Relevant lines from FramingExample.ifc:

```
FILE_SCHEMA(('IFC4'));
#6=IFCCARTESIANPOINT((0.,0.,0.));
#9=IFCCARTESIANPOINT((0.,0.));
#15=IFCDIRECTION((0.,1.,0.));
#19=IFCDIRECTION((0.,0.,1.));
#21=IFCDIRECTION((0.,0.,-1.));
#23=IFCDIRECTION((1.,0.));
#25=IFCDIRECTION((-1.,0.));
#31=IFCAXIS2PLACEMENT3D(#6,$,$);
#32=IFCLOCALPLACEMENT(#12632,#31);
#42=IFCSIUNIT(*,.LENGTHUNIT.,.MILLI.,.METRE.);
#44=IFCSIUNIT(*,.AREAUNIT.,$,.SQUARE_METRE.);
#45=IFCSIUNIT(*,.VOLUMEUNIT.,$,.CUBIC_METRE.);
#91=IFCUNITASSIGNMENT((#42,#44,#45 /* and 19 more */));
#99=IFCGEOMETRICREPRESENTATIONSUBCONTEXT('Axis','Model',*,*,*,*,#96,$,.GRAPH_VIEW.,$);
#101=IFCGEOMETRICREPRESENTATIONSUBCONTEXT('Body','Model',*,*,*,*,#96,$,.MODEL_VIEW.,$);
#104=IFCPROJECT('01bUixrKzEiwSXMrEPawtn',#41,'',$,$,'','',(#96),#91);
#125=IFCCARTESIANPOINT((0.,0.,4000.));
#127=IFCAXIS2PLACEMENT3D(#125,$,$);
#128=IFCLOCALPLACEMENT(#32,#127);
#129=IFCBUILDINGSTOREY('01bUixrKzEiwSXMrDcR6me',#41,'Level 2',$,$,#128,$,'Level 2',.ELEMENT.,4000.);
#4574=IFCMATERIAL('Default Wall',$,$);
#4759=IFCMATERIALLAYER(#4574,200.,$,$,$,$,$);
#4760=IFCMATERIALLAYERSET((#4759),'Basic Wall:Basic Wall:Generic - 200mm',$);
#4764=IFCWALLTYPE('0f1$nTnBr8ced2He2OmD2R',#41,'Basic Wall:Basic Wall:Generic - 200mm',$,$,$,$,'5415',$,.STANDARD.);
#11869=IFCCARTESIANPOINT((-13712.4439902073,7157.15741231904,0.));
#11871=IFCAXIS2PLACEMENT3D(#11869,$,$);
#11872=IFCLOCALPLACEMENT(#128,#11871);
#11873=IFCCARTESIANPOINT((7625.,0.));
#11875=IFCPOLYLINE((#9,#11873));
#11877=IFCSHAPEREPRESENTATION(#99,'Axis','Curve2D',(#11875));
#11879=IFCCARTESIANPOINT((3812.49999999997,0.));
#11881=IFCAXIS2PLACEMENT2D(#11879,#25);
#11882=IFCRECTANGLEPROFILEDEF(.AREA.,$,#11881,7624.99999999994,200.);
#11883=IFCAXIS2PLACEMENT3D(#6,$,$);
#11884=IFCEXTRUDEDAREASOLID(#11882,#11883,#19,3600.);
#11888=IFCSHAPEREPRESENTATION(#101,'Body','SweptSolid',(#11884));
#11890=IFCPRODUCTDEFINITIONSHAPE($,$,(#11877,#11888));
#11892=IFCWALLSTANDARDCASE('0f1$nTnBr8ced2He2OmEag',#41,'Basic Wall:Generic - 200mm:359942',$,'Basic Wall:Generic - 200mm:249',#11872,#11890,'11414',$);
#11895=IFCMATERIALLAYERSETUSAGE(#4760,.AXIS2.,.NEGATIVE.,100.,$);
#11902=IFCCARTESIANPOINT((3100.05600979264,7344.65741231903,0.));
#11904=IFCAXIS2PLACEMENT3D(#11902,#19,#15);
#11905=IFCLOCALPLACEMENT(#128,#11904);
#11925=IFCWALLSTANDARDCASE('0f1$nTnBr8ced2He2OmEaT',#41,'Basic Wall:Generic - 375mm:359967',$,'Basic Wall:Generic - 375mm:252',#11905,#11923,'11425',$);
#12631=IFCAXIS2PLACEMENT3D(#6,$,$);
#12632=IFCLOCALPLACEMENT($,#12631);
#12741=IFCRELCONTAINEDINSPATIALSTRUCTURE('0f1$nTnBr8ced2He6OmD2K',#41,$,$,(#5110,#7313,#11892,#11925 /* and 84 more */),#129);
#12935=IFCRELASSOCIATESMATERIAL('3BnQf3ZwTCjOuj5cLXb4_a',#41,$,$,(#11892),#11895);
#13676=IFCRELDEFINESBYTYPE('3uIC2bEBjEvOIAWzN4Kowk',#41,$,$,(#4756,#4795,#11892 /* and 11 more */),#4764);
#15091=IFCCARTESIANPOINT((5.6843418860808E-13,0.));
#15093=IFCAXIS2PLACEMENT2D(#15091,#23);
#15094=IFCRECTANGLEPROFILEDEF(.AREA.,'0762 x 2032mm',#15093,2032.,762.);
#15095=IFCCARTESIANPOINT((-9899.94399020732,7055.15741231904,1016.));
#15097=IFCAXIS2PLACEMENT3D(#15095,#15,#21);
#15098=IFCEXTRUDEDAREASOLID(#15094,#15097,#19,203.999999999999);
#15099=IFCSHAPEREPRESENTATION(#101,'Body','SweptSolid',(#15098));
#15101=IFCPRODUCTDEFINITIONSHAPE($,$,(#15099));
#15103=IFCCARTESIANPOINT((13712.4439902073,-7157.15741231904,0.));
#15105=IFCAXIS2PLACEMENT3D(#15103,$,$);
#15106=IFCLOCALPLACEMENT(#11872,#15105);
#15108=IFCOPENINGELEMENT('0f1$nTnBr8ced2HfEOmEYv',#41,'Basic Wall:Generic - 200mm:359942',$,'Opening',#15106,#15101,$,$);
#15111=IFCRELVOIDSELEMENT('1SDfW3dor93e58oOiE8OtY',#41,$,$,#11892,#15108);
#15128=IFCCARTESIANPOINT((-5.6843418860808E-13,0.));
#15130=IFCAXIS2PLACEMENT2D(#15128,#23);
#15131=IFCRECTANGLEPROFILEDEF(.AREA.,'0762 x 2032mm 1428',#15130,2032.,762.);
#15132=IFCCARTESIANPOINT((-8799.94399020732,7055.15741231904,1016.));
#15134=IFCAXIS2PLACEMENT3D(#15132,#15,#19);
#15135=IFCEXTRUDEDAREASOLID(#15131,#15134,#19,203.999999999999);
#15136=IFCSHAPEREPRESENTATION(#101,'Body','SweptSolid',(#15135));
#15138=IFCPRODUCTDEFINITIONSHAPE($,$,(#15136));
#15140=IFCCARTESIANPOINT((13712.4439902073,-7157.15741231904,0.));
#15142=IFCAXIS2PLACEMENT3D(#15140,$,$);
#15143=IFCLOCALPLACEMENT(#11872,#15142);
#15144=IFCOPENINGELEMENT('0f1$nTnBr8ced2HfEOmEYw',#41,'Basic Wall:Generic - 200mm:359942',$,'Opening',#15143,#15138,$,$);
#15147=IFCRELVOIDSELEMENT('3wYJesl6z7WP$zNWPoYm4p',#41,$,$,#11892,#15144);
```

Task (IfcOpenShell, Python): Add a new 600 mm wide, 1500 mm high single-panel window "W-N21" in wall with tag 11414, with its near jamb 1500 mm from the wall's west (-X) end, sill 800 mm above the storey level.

```python
import numpy as np
import ifcopenshell
import ifcopenshell.api.feature
import ifcopenshell.api.geometry
import ifcopenshell.api.root
import ifcopenshell.api.spatial
import ifcopenshell.geom
import ifcopenshell.util.element
import ifcopenshell.util.placement
import ifcopenshell.util.representation
import ifcopenshell.util.shape
import ifcopenshell.util.unit

model = ifcopenshell.open("FramingExample.ifc")
unit_scale = ifcopenshell.util.unit.calculate_unit_scale(model)
settings = ifcopenshell.geom.settings()


def volume(element):
    """Net volume in cubic metres, openings subtracted."""
    shape = ifcopenshell.geom.create_shape(settings, element)
    return ifcopenshell.util.shape.get_volume(shape.geometry)


wall = model.by_guid("0f1$nTnBr8ced2He2OmEag")
storey = ifcopenshell.util.element.get_container(wall, ifc_class="IfcBuildingStorey")
context = ifcopenshell.util.representation.get_context(model, "Model", "Body", "MODEL_VIEW")
before = volume(wall)

width, height, from_end, sill = 0.6, 1.5, 1.5, 0.8  # metres

# The wall runs along its own X axis, and the end named is its -X end.
wall_shape = ifcopenshell.geom.create_shape(settings, wall)
x, y, z = ifcopenshell.util.shape.get_vertices(wall_shape.geometry).T
start = x.min() + from_end
face, thickness = float(y.min()), float(y.max() - y.min())
wall_matrix = ifcopenshell.util.placement.get_local_placement(wall.ObjectPlacement)
level = ifcopenshell.util.placement.get_local_placement(storey.ObjectPlacement)[2, 3]


def in_wall(x, y):
    """Placement at x, y metres in the wall's axes, at sill height."""
    matrix = wall_matrix.copy()
    matrix[:, 3] = wall_matrix @ np.array([x / unit_scale, y / unit_scale, 0.0, 1.0])
    matrix[2, 3] = level + sill / unit_scale
    return matrix


# Opening: a box that overshoots both wall faces by 50 mm.
opening = ifcopenshell.api.root.create_entity(model, ifc_class="IfcOpeningElement", predefined_type="OPENING")
box = ifcopenshell.api.geometry.add_wall_representation(
    model, context=context, length=width, height=height, thickness=thickness + 0.1
)
ifcopenshell.api.geometry.assign_representation(model, product=opening, representation=box)
ifcopenshell.api.geometry.edit_object_placement(model, product=opening, matrix=in_wall(start, face - 0.05), is_si=False)
ifcopenshell.api.feature.add_feature(model, feature=opening, element=wall)

window = ifcopenshell.api.root.create_entity(model, ifc_class="IfcWindow", name="W-N21", predefined_type="WINDOW")
window.OverallWidth, window.OverallHeight = width / unit_scale, height / unit_scale
window.PartitioningType = "SINGLE_PANEL"
body = ifcopenshell.api.geometry.add_window_representation(
    model,
    context=context,
    overall_width=window.OverallWidth,
    overall_height=window.OverallHeight,
    partition_type="SINGLE_PANEL",
)
ifcopenshell.api.geometry.assign_representation(model, product=window, representation=body)
ifcopenshell.api.spatial.assign_container(model, products=[window], relating_structure=storey)
ifcopenshell.api.feature.add_filling(model, opening=opening, element=window)

# Centre the window in the wall's thickness.
ifcopenshell.api.geometry.edit_object_placement(model, product=window, matrix=in_wall(start, face), is_si=False)
window_shape = ifcopenshell.geom.create_shape(settings, window)
depth = ifcopenshell.util.shape.get_vertices(window_shape.geometry)[:, 1]
offset = face + thickness / 2 - (depth.min() + depth.max()) / 2
ifcopenshell.api.geometry.edit_object_placement(model, product=window, matrix=in_wall(start, offset), is_si=False)

after = volume(wall)

print(f"wall volume {before:.3f} -> {after:.3f} m3")

model.write("FramingExample-out.ifc")
```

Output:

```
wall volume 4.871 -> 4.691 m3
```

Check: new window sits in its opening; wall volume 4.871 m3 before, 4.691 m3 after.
